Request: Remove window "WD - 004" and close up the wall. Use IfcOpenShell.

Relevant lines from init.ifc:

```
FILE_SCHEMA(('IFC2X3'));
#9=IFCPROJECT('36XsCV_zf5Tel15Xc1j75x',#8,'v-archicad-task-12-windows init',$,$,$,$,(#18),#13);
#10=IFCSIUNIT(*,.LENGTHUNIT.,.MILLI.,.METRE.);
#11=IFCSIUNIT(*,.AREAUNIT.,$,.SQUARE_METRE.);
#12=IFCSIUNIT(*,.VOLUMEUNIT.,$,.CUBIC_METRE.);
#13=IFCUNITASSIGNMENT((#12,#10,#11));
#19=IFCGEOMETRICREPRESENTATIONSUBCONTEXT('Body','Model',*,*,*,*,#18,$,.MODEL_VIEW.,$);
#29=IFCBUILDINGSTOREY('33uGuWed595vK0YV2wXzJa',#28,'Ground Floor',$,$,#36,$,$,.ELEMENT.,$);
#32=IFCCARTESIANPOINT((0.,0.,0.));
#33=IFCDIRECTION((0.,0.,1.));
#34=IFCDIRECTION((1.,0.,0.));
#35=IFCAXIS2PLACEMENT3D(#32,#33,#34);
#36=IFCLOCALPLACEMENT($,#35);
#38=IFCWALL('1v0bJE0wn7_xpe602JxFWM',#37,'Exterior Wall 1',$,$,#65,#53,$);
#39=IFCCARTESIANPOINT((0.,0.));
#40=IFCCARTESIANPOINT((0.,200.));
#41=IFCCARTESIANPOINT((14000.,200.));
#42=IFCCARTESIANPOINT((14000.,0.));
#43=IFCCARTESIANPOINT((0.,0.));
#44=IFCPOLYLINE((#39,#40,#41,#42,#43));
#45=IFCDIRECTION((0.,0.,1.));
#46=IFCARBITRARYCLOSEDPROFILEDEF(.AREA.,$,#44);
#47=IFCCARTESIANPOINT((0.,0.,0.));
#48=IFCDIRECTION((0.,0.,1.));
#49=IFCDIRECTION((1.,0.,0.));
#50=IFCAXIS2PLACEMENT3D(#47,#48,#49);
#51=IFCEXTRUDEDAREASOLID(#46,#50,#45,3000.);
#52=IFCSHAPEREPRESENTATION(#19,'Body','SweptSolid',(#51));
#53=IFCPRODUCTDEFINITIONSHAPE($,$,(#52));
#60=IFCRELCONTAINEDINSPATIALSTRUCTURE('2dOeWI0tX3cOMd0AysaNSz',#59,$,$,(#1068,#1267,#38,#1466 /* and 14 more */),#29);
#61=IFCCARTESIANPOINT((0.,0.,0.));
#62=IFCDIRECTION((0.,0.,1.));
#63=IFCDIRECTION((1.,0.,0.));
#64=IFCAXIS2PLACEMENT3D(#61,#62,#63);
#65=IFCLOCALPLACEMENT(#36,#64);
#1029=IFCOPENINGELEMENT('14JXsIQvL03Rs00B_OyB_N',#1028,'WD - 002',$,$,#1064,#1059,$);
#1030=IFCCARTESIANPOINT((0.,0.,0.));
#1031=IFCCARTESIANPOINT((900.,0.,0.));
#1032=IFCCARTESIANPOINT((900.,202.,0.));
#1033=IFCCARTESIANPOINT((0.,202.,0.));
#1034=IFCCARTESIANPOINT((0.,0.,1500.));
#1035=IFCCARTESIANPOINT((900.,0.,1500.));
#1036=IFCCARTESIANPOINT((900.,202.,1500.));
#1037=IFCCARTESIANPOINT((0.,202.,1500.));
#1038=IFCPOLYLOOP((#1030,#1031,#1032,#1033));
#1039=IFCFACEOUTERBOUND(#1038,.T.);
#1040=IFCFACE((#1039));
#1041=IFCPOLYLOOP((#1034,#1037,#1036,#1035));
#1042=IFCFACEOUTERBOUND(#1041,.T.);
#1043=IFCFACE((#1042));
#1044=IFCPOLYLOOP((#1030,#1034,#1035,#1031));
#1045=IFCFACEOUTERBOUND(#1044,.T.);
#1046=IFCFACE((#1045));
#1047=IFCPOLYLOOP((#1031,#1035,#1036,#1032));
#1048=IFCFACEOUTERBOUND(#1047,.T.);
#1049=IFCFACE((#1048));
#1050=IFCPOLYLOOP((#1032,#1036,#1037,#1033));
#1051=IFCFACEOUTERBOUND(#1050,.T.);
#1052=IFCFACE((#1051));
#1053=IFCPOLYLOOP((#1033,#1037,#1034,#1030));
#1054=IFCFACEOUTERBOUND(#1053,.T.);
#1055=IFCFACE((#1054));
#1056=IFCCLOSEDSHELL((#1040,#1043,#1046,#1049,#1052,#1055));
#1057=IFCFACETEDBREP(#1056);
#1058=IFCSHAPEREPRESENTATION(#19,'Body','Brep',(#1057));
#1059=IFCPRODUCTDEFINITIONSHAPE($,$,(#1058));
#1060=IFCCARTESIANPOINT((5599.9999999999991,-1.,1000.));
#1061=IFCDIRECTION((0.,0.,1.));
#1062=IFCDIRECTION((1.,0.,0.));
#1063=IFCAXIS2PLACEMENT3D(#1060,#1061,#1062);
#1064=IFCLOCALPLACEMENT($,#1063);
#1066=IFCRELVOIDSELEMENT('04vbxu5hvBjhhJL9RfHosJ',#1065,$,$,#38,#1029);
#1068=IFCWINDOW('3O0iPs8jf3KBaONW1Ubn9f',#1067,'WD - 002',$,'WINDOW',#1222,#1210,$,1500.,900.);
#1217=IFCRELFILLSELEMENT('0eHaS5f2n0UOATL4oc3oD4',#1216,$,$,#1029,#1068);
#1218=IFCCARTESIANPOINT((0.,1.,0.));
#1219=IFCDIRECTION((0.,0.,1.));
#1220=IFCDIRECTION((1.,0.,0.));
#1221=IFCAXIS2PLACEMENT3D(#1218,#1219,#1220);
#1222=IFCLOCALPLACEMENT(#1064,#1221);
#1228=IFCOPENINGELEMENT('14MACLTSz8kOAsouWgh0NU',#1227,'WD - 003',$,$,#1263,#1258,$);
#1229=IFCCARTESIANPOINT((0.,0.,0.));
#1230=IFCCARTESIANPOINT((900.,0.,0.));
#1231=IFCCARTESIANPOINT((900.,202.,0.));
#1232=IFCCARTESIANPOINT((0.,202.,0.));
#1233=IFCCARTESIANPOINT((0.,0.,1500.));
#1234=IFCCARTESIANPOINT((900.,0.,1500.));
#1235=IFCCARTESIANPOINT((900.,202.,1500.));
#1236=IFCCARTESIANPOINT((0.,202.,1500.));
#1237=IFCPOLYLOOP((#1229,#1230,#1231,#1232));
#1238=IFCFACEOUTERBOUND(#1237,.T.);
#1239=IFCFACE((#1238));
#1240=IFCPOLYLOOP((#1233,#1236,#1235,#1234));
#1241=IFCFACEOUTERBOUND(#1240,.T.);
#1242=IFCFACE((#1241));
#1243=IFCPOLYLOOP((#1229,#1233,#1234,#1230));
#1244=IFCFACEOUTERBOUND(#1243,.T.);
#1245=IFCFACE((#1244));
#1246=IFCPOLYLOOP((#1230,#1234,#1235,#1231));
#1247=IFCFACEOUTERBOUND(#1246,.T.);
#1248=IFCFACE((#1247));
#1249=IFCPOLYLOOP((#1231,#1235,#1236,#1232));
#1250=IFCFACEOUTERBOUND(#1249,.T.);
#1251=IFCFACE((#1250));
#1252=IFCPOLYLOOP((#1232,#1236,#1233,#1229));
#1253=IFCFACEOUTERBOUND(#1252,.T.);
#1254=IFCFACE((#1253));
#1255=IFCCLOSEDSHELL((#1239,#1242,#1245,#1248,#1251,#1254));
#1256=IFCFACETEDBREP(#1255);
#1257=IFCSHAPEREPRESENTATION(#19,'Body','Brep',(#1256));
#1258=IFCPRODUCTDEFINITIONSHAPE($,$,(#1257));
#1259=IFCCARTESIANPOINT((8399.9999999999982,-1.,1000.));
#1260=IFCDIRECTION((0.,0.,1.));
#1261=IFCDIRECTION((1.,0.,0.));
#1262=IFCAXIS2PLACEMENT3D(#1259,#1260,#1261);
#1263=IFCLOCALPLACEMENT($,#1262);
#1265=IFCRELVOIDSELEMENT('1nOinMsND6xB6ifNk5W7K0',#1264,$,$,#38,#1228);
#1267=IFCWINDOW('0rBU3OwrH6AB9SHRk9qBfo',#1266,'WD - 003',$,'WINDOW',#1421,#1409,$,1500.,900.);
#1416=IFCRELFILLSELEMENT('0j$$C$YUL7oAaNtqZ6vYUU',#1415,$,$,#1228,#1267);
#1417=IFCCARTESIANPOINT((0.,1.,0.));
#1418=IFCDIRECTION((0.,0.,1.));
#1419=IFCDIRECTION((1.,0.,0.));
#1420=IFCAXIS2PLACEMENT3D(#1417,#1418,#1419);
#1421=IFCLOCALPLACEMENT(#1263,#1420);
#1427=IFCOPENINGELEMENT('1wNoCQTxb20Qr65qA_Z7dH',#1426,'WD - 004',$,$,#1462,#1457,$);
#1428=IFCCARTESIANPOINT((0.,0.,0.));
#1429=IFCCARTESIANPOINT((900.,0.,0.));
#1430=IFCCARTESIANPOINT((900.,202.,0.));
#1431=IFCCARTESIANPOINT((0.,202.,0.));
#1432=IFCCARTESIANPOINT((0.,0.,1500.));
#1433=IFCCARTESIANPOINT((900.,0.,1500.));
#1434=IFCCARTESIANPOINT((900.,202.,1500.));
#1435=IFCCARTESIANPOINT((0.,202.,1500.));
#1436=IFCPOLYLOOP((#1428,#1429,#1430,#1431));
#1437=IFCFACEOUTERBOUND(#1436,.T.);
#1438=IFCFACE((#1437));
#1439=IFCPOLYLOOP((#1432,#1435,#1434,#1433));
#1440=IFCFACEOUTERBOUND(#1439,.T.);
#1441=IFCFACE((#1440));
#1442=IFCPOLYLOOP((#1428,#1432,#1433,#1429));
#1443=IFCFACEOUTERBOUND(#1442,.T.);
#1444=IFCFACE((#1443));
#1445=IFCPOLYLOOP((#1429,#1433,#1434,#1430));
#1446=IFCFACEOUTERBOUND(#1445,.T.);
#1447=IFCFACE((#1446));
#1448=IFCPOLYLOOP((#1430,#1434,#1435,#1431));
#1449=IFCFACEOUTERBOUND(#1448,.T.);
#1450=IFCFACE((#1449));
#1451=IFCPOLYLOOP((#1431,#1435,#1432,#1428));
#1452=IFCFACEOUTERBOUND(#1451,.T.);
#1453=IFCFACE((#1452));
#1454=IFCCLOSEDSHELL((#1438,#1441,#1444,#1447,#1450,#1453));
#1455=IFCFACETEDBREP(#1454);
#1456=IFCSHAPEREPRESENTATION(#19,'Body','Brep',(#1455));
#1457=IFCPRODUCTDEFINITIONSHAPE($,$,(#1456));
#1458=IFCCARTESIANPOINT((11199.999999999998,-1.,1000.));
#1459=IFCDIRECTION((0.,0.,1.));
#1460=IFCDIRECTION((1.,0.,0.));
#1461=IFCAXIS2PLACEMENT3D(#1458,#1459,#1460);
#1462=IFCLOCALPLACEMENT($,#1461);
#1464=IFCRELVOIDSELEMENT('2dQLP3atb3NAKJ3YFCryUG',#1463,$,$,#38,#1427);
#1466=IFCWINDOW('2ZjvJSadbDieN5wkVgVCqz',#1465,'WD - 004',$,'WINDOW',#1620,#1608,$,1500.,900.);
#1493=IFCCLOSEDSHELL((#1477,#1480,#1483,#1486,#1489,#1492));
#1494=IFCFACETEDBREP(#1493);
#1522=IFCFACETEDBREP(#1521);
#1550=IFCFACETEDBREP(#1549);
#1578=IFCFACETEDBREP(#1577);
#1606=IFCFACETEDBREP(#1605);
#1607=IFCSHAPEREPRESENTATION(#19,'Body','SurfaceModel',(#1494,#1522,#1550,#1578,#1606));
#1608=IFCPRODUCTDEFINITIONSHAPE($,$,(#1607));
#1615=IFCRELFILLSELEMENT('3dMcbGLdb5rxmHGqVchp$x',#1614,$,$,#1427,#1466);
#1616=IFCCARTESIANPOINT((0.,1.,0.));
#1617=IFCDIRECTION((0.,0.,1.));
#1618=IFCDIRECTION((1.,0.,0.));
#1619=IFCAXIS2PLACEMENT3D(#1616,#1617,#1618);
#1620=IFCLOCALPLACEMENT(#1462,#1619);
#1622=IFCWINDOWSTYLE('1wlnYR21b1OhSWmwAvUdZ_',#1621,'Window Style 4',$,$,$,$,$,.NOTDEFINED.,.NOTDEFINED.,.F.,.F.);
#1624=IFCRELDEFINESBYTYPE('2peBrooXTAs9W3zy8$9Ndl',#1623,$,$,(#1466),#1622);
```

```python
import ifcopenshell
import ifcopenshell.api.feature
import ifcopenshell.api.root
import ifcopenshell.geom
import ifcopenshell.util.shape

model = ifcopenshell.open("init.ifc")
settings = ifcopenshell.geom.settings()


def volume(element):
    """Net volume in cubic metres, openings subtracted."""
    shape = ifcopenshell.geom.create_shape(settings, element)
    return ifcopenshell.util.shape.get_volume(shape.geometry)


window = model.by_guid("2ZjvJSadbDieN5wkVgVCqz")
opening = window.FillsVoids[0].RelatingOpeningElement
wall = opening.VoidsElements[0].RelatingBuildingElement
before = volume(wall)

ifcopenshell.api.root.remove_product(model, product=window)
ifcopenshell.api.feature.remove_feature(model, feature=opening)

after = volume(wall)

print(f"wall volume {before:.3f} -> {after:.3f} m3")

model.write("init-out.ifc")
```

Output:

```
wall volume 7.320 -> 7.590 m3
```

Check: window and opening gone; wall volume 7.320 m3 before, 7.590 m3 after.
